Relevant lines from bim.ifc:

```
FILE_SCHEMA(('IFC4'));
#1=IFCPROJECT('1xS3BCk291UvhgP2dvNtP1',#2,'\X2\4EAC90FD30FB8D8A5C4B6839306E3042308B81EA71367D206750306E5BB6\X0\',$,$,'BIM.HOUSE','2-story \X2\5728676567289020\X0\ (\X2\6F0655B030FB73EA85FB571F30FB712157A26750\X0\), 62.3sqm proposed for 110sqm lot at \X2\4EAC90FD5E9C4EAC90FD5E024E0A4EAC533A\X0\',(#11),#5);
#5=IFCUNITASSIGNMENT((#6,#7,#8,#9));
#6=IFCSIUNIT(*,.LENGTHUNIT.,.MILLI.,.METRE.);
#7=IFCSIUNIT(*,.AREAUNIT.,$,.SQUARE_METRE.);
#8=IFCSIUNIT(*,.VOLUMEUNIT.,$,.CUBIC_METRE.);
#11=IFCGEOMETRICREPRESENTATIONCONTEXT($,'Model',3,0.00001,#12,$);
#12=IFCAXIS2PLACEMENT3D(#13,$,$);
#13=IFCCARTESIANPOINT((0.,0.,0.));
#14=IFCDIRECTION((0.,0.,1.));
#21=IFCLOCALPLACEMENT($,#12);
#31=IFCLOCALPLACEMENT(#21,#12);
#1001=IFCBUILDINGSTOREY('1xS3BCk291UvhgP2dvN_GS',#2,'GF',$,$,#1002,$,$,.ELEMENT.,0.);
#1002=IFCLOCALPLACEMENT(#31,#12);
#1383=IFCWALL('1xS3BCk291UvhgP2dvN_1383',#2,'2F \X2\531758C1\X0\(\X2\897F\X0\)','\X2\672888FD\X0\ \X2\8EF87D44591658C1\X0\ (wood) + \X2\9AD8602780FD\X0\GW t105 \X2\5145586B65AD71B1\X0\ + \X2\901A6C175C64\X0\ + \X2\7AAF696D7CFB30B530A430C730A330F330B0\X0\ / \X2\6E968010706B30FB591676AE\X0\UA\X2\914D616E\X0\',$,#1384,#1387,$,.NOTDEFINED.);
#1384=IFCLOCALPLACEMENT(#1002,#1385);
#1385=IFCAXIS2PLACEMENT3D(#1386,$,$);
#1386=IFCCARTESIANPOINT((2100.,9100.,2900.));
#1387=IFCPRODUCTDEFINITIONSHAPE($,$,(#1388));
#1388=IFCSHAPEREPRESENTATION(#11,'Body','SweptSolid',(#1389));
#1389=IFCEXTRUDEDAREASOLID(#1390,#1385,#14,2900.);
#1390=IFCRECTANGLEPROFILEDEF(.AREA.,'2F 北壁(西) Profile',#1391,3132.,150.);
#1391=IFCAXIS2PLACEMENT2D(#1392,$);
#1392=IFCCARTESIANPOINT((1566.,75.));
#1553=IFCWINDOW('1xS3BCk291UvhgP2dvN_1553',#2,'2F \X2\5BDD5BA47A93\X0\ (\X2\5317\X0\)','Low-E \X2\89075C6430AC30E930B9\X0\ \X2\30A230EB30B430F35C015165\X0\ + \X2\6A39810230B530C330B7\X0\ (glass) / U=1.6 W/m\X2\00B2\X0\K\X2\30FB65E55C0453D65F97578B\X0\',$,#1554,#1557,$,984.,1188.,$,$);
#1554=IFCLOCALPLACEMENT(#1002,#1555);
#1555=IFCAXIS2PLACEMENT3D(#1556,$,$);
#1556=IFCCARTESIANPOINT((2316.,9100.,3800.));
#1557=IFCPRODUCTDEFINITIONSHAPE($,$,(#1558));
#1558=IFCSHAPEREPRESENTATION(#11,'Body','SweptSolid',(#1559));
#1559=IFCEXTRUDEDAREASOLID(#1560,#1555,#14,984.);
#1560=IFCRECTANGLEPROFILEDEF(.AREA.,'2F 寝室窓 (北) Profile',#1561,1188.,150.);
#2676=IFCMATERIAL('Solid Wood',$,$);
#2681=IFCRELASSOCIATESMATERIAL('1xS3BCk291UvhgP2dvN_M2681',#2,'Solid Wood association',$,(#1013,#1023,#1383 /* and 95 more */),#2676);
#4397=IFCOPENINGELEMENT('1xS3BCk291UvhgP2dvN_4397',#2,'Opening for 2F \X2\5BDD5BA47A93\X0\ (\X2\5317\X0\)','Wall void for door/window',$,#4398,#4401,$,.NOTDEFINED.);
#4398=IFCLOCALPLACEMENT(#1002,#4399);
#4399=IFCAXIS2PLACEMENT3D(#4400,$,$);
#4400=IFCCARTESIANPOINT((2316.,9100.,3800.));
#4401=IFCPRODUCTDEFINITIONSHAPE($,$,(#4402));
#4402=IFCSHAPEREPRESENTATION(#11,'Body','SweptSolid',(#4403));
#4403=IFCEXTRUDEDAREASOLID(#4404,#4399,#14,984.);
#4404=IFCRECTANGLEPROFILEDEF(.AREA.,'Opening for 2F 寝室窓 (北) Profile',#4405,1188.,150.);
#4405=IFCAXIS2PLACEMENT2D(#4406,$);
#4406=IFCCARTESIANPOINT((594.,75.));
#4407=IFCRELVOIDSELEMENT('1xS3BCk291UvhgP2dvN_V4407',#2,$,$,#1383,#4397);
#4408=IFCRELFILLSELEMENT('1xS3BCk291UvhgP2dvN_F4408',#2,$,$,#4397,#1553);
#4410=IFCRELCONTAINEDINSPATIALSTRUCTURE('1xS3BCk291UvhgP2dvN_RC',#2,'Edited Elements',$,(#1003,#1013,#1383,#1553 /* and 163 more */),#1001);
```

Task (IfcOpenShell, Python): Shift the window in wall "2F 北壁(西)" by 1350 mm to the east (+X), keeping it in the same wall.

```python
import ifcopenshell
import ifcopenshell.api.geometry
import ifcopenshell.util.placement

model = ifcopenshell.open("bim.ifc")

window = model.by_guid("1xS3BCk291UvhgP2dvN_1553")
opening = window.FillsVoids[0].RelatingOpeningElement
wall = opening.VoidsElements[0].RelatingBuildingElement

wall_matrix = ifcopenshell.util.placement.get_local_placement(wall.ObjectPlacement)
shift = wall_matrix[:3, 0] * 1350.0
before = ifcopenshell.util.placement.get_local_placement(window.ObjectPlacement)[:3, 3].copy()

# The window is not placed relative to its opening, so move both.
for product in (opening, window):
    matrix = ifcopenshell.util.placement.get_local_placement(product.ObjectPlacement)
    matrix[:3, 3] += shift
    ifcopenshell.api.geometry.edit_object_placement(model, product=product, matrix=matrix, is_si=False)

after = ifcopenshell.util.placement.get_local_placement(window.ObjectPlacement)[:3, 3]
print("window moved by", (after - before).round(3) + 0.0)

model.write("bim_edited.ifc")
```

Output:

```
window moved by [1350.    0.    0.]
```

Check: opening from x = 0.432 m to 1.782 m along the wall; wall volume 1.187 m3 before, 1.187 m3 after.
